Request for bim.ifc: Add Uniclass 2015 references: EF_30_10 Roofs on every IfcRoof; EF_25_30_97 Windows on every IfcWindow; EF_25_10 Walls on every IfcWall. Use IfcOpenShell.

First a look at what the model holds.

```python
import ifcopenshell

model = ifcopenshell.open("bim.ifc")
print(model.schema)
print("classifications:", [c.Name for c in model.by_type("IfcClassification")])
for ifc_class in ("IfcDoor", "IfcRoof", "IfcStair", "IfcWall", "IfcWindow"):
    print(ifc_class, len(model.by_type(ifc_class)))
```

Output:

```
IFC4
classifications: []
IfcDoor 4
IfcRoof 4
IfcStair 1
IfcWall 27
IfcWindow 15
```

```python
import ifcopenshell
import ifcopenshell.api.classification

model = ifcopenshell.open("bim.ifc")

system = ifcopenshell.api.classification.add_classification(model, classification="Uniclass 2015")

codes = {
    "IfcRoof": ("EF_30_10", "Roofs"),
    "IfcWindow": ("EF_25_30_97", "Windows"),
    "IfcWall": ("EF_25_10", "Walls"),
}
for ifc_class, (code, name) in codes.items():
    products = model.by_type(ifc_class)
    ifcopenshell.api.classification.add_reference(
        model, products=products, classification=system, identification=code, name=name
    )
    print(code, len(products))

model.write("bim_rev.ifc")
```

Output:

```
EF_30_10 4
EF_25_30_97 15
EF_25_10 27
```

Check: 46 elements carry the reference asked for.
